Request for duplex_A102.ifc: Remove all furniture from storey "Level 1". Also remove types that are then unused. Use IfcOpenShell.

First a look at what the model holds.

```python
import ifcopenshell
import ifcopenshell.util.element

model = ifcopenshell.open("duplex_A102.ifc")
print(model.schema)
storey = next(s for s in model.by_type("IfcBuildingStorey") if s.Name == "Level 1")
furniture = [e for e in ifcopenshell.util.element.get_decomposition(storey) if e.is_a("IfcFurnishingElement")]
seen = {}
for e in furniture:
    element_type = ifcopenshell.util.element.get_type(e)
    name = element_type.Name if element_type not in (None, e) else None
    seen[name] = seen.get(name, 0) + 1
for name, count in sorted(seen.items(), key=str):
    print(count, "x", name)
```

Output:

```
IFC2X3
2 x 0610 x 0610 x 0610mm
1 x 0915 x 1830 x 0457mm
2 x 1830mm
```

```python
import ifcopenshell
import ifcopenshell.api.root
import ifcopenshell.util.element

model = ifcopenshell.open("duplex_A102.ifc")

storey = next(s for s in model.by_type("IfcBuildingStorey") if s.Name == "Level 1")
furniture = [e for e in ifcopenshell.util.element.get_decomposition(storey) if e.is_a("IfcFurnishingElement")]
types = {ifcopenshell.util.element.get_type(e) for e in furniture} - {None, *furniture}

for e in furniture:
    ifcopenshell.api.root.remove_product(model, product=e)
print(len(furniture), "removed")

unused = [t for t in types if not ifcopenshell.util.element.get_types(t)]
for t in unused:
    ifcopenshell.api.root.remove_product(model, product=t)
print(len(unused), "unused types removed")

model.write("duplex_A102_rev.ifc")
```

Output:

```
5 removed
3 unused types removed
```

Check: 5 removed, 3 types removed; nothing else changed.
